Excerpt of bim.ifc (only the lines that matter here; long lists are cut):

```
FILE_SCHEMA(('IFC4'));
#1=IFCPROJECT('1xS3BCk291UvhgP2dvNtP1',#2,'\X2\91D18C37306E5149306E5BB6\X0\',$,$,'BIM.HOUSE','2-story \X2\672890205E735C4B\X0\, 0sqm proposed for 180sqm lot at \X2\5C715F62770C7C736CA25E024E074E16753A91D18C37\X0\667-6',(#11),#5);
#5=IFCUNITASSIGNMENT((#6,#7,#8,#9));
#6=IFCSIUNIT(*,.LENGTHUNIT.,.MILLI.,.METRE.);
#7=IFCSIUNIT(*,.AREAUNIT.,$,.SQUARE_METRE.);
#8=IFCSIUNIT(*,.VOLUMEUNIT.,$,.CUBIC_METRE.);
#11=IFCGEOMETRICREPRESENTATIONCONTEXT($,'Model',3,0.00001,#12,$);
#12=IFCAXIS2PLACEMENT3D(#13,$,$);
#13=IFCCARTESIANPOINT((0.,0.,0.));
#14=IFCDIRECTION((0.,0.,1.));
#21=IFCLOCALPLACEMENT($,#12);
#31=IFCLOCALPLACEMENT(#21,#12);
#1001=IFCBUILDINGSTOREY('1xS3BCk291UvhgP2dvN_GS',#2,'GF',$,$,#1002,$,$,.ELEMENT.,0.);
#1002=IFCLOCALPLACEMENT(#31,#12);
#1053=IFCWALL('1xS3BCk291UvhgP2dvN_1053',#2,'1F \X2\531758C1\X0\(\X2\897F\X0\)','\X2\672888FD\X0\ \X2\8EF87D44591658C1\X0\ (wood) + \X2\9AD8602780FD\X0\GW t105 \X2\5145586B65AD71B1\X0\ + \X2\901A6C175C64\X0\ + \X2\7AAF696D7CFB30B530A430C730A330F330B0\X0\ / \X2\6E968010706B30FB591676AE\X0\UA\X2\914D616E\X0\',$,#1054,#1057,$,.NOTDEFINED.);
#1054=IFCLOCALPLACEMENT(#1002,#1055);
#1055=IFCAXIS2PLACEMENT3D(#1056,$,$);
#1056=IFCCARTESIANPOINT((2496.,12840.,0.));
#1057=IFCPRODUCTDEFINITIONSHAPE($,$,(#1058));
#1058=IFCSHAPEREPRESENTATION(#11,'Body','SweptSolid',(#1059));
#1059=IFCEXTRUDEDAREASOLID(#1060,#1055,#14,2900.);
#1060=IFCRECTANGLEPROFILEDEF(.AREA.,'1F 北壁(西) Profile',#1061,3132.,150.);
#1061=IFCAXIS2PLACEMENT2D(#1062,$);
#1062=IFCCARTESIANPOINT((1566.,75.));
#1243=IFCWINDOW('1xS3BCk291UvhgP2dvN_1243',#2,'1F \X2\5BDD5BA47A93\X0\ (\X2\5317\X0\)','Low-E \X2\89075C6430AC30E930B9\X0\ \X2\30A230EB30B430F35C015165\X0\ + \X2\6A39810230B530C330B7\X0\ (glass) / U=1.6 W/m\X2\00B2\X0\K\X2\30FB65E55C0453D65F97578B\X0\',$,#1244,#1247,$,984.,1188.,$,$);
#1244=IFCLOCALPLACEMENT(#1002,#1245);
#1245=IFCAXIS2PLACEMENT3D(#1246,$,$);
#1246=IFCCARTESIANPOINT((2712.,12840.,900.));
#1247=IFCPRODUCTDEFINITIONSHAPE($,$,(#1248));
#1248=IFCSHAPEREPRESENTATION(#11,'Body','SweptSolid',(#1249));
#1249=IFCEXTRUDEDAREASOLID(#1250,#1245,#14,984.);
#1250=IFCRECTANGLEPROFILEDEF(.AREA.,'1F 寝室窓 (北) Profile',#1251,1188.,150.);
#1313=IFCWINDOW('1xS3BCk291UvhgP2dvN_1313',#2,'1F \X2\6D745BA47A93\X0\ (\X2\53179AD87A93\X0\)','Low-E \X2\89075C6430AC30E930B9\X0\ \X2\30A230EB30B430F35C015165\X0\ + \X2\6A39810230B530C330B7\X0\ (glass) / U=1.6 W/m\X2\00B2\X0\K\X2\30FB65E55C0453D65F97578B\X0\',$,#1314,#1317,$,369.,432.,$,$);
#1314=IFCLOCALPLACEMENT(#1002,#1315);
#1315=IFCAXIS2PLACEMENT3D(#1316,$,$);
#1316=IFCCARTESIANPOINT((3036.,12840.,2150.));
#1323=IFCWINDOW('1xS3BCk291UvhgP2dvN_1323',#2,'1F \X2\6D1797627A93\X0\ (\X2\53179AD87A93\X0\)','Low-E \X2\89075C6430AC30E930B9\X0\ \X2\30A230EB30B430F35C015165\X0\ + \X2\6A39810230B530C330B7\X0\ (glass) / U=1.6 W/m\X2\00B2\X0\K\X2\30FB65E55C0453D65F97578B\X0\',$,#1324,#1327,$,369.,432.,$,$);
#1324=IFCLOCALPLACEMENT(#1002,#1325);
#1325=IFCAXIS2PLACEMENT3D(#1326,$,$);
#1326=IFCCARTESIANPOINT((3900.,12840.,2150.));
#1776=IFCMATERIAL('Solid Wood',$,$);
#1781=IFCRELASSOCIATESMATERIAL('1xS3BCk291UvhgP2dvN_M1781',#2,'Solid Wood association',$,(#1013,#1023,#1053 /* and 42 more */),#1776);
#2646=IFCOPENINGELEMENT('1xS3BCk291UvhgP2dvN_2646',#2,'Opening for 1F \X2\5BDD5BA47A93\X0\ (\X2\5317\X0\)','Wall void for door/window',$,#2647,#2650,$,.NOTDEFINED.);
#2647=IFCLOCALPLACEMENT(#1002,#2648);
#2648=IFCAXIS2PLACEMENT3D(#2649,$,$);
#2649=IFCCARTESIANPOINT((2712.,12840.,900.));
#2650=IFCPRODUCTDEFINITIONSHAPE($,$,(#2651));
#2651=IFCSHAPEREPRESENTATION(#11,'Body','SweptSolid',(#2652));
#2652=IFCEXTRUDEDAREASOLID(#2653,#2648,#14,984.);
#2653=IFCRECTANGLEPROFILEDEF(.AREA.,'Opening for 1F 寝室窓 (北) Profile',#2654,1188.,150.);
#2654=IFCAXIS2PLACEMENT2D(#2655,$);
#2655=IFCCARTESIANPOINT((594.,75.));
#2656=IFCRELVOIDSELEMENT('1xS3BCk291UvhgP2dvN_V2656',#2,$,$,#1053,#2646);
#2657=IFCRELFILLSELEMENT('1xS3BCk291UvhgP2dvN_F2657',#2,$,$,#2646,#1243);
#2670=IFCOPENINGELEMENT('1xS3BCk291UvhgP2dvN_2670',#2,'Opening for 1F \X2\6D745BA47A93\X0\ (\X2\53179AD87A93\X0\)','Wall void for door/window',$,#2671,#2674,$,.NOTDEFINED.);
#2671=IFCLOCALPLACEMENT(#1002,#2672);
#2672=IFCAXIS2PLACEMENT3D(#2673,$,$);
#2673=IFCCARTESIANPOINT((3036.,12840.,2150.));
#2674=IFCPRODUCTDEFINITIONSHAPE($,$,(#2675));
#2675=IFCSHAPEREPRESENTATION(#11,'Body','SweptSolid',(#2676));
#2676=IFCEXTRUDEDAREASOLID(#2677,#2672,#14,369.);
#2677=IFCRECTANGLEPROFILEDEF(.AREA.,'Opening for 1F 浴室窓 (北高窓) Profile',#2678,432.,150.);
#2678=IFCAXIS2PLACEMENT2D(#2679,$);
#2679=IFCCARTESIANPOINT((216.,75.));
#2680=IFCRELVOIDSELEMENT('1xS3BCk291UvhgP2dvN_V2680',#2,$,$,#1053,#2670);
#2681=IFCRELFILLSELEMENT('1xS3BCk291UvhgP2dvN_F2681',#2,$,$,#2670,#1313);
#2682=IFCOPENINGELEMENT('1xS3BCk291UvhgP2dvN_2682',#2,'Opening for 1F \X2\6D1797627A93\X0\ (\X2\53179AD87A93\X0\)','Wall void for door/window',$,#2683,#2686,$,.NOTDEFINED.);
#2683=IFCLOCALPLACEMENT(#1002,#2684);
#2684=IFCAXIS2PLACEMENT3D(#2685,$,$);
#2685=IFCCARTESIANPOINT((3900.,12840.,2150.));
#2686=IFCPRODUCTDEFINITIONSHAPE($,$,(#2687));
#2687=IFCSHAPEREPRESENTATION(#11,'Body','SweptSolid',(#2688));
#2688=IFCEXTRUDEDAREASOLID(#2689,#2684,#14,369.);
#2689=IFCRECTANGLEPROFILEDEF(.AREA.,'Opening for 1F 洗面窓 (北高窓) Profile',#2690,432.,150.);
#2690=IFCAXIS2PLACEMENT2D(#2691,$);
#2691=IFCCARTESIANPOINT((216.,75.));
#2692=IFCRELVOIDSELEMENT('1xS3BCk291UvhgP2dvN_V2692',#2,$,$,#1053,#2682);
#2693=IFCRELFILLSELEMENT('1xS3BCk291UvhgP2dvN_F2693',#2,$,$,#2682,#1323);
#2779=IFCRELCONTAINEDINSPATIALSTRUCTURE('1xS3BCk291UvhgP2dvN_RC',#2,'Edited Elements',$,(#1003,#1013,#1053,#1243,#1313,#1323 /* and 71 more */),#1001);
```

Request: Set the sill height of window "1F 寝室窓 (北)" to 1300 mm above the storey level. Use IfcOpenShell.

```python
import numpy as np
import ifcopenshell
import ifcopenshell.api.geometry
import ifcopenshell.geom
import ifcopenshell.util.element
import ifcopenshell.util.placement
import ifcopenshell.util.shape
import ifcopenshell.util.unit

model = ifcopenshell.open("bim.ifc")
unit_scale = ifcopenshell.util.unit.calculate_unit_scale(model)

window = model.by_guid("1xS3BCk291UvhgP2dvN_1243")
opening = window.FillsVoids[0].RelatingOpeningElement
storey = ifcopenshell.util.element.get_container(window, ifc_class="IfcBuildingStorey")
level = ifcopenshell.util.placement.get_local_placement(storey.ObjectPlacement)[2, 3]

# The opening's origin need not be at the sill, so measure its lowest point.
shape = ifcopenshell.geom.create_shape(ifcopenshell.geom.settings(), opening)
bottom = ifcopenshell.util.shape.get_shape_bottom_elevation(shape, shape.geometry) / unit_scale
dz = level + 1.3 / unit_scale - bottom

shift = np.array([0.0, 0.0, dz])
# The window is not placed relative to its opening, so move both.
for product in (opening, window):
    matrix = ifcopenshell.util.placement.get_local_placement(product.ObjectPlacement)
    matrix[:3, 3] += shift
    ifcopenshell.api.geometry.edit_object_placement(model, product=product, matrix=matrix, is_si=False)

print(f"moved by {dz * unit_scale:+.3f} m")

model.write("bim-out.ifc")
```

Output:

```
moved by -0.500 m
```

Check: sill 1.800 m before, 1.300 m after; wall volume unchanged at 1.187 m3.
